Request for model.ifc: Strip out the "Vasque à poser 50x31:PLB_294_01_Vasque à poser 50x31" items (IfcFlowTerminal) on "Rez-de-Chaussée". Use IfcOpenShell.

First a look at what the model holds.

```python
import ifcopenshell
import ifcopenshell.util.element

model = ifcopenshell.open("model.ifc")
print(model.schema)
storey = next(s for s in model.by_type("IfcBuildingStorey") if s.Name == "Rez-de-Chaussée")
terminals = [e for e in ifcopenshell.util.element.get_decomposition(storey) if e.is_a("IfcFlowTerminal")]
seen = {}
for e in terminals:
    element_type = ifcopenshell.util.element.get_type(e)
    name = element_type.Name if element_type not in (None, e) else None
    seen[name] = seen.get(name, 0) + 1
for name, count in sorted(seen.items(), key=str):
    print(count, "x", name)
```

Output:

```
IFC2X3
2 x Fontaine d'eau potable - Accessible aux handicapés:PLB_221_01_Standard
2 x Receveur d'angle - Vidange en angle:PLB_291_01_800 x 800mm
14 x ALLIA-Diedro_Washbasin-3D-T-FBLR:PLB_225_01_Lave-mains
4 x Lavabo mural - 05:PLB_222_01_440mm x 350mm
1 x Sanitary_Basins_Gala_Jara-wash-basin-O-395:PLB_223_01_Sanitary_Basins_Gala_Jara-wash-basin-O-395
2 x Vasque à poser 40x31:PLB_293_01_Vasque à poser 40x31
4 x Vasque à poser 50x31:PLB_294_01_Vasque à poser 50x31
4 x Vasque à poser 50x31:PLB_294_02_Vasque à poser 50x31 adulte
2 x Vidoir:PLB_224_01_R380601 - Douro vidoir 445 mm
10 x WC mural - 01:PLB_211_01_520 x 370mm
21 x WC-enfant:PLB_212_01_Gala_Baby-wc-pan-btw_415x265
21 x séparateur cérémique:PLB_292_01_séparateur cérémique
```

```python
import ifcopenshell
import ifcopenshell.api.root
import ifcopenshell.util.element

model = ifcopenshell.open("model.ifc")

storey = next(s for s in model.by_type("IfcBuildingStorey") if s.Name == "Rez-de-Chaussée")
terminals = [e for e in ifcopenshell.util.element.get_decomposition(storey) if e.is_a("IfcFlowTerminal")]
targets = [e for e in terminals if (t := ifcopenshell.util.element.get_type(e)) not in (None, e) and t.Name == "Vasque à poser 50x31:PLB_294_01_Vasque à poser 50x31"]

for e in targets:
    ifcopenshell.api.root.remove_product(model, product=e)
print(len(targets), "removed")

model.write("model_rev.ifc")
```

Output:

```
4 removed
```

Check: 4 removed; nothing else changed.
